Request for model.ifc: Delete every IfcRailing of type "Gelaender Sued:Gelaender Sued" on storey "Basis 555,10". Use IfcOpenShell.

First a look at what the model holds.

```python
import ifcopenshell
import ifcopenshell.util.element

model = ifcopenshell.open("model.ifc")
print(model.schema)
storey = next(s for s in model.by_type("IfcBuildingStorey") if s.Name == "Basis 555,10")
railings = [e for e in ifcopenshell.util.element.get_decomposition(storey) if e.is_a("IfcRailing")]
seen = {}
for e in railings:
    element_type = ifcopenshell.util.element.get_type(e)
    name = element_type.Name if element_type not in (None, e) else None
    seen[name] = seen.get(name, 0) + 1
for name, count in sorted(seen.items(), key=str):
    print(count, "x", name)
```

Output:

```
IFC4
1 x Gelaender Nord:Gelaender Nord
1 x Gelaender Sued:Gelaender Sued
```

```python
import ifcopenshell
import ifcopenshell.api.root
import ifcopenshell.util.element

model = ifcopenshell.open("model.ifc")

storey = next(s for s in model.by_type("IfcBuildingStorey") if s.Name == "Basis 555,10")
railings = [e for e in ifcopenshell.util.element.get_decomposition(storey) if e.is_a("IfcRailing")]
targets = [e for e in railings if (t := ifcopenshell.util.element.get_type(e)) not in (None, e) and t.Name == "Gelaender Sued:Gelaender Sued"]

for e in targets:
    ifcopenshell.api.root.remove_product(model, product=e)
print(len(targets), "removed")

model.write("model_rev.ifc")
```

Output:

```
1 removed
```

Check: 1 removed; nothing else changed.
